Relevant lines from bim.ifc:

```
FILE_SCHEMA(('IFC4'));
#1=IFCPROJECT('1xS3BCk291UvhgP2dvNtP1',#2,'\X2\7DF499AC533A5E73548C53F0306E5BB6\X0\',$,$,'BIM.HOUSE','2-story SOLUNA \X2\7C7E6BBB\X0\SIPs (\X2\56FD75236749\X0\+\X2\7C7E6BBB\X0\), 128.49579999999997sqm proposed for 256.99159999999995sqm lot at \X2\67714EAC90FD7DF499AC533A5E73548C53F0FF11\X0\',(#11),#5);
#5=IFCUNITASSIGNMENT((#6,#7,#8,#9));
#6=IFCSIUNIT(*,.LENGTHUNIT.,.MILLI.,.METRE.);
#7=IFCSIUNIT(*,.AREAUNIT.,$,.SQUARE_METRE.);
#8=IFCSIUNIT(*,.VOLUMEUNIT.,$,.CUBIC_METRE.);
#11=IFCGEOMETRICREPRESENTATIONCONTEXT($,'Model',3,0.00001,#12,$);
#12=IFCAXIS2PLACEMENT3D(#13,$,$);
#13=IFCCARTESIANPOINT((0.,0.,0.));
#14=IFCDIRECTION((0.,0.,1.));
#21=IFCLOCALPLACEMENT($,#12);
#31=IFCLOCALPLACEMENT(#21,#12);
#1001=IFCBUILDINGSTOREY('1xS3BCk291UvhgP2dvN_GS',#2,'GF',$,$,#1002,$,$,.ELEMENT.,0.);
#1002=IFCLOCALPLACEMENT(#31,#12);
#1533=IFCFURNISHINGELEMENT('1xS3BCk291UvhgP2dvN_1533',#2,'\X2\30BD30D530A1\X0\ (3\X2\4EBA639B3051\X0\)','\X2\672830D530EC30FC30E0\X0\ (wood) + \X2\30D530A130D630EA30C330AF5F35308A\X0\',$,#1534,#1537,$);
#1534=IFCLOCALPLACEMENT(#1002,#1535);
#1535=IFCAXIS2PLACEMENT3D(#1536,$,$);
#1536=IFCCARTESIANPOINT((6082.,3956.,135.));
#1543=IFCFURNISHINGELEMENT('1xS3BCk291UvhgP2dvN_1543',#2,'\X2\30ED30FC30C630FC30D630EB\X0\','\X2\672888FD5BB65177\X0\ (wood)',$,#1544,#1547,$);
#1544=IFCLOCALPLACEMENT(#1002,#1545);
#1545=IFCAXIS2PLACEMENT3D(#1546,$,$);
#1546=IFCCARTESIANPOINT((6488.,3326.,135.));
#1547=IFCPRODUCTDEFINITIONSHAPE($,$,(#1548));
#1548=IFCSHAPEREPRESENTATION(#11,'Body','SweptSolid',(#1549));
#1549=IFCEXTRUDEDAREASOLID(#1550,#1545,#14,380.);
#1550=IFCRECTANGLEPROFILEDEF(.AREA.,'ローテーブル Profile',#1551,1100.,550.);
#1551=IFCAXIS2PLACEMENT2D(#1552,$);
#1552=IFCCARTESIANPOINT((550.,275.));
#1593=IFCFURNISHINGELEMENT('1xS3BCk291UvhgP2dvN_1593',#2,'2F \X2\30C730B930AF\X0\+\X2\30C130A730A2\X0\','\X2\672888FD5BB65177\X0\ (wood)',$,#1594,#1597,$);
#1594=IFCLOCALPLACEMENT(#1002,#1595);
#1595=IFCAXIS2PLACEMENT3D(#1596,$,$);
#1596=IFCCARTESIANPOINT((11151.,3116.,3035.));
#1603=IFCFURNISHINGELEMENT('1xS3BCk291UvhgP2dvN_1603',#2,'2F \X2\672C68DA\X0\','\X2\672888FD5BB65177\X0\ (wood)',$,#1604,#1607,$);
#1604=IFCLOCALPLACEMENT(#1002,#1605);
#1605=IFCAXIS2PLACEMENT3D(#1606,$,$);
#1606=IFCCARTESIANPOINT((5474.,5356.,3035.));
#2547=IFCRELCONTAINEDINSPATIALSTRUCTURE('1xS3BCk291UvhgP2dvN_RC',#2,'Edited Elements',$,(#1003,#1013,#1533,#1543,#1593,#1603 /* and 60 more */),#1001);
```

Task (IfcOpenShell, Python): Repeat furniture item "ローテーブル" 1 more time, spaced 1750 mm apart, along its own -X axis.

```python
import ifcopenshell
import ifcopenshell.api.geometry
import ifcopenshell.api.root
import ifcopenshell.util.element
import ifcopenshell.util.placement
import ifcopenshell.util.unit

model = ifcopenshell.open("bim.ifc")
unit_scale = ifcopenshell.util.unit.calculate_unit_scale(model)


def reuse_history(source, copy):
    """copy_class also copies each property set's owner history, people and application; keep the originals."""
    for rel in copy.IsDefinedBy:
        if rel.is_a("IfcRelDefinesByProperties") and (history := rel.RelatingPropertyDefinition.OwnerHistory):
            rel.RelatingPropertyDefinition.OwnerHistory = source.OwnerHistory
            ifcopenshell.util.element.remove_deep2(model, history)


source = model.by_guid("1xS3BCk291UvhgP2dvN_1543")
base = ifcopenshell.util.placement.get_local_placement(source.ObjectPlacement)
step = -base[:3, 0] * 1.75 / unit_scale

for i in range(1, 2):
    copy = ifcopenshell.api.root.copy_class(model, product=source)
    copy.Representation = ifcopenshell.util.element.copy_deep(
        model, source.Representation, exclude=["IfcGeometricRepresentationContext", "IfcRepresentationMap"]
    )
    reuse_history(source, copy)
    matrix = base.copy()
    matrix[:3, 3] += i * step
    print("added at", matrix[:3, 3].round(3) + 0.0)
    ifcopenshell.api.geometry.edit_object_placement(model, product=copy, matrix=matrix, is_si=False)

model.write("bim_v2.ifc")
```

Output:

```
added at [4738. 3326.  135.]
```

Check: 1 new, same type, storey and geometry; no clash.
